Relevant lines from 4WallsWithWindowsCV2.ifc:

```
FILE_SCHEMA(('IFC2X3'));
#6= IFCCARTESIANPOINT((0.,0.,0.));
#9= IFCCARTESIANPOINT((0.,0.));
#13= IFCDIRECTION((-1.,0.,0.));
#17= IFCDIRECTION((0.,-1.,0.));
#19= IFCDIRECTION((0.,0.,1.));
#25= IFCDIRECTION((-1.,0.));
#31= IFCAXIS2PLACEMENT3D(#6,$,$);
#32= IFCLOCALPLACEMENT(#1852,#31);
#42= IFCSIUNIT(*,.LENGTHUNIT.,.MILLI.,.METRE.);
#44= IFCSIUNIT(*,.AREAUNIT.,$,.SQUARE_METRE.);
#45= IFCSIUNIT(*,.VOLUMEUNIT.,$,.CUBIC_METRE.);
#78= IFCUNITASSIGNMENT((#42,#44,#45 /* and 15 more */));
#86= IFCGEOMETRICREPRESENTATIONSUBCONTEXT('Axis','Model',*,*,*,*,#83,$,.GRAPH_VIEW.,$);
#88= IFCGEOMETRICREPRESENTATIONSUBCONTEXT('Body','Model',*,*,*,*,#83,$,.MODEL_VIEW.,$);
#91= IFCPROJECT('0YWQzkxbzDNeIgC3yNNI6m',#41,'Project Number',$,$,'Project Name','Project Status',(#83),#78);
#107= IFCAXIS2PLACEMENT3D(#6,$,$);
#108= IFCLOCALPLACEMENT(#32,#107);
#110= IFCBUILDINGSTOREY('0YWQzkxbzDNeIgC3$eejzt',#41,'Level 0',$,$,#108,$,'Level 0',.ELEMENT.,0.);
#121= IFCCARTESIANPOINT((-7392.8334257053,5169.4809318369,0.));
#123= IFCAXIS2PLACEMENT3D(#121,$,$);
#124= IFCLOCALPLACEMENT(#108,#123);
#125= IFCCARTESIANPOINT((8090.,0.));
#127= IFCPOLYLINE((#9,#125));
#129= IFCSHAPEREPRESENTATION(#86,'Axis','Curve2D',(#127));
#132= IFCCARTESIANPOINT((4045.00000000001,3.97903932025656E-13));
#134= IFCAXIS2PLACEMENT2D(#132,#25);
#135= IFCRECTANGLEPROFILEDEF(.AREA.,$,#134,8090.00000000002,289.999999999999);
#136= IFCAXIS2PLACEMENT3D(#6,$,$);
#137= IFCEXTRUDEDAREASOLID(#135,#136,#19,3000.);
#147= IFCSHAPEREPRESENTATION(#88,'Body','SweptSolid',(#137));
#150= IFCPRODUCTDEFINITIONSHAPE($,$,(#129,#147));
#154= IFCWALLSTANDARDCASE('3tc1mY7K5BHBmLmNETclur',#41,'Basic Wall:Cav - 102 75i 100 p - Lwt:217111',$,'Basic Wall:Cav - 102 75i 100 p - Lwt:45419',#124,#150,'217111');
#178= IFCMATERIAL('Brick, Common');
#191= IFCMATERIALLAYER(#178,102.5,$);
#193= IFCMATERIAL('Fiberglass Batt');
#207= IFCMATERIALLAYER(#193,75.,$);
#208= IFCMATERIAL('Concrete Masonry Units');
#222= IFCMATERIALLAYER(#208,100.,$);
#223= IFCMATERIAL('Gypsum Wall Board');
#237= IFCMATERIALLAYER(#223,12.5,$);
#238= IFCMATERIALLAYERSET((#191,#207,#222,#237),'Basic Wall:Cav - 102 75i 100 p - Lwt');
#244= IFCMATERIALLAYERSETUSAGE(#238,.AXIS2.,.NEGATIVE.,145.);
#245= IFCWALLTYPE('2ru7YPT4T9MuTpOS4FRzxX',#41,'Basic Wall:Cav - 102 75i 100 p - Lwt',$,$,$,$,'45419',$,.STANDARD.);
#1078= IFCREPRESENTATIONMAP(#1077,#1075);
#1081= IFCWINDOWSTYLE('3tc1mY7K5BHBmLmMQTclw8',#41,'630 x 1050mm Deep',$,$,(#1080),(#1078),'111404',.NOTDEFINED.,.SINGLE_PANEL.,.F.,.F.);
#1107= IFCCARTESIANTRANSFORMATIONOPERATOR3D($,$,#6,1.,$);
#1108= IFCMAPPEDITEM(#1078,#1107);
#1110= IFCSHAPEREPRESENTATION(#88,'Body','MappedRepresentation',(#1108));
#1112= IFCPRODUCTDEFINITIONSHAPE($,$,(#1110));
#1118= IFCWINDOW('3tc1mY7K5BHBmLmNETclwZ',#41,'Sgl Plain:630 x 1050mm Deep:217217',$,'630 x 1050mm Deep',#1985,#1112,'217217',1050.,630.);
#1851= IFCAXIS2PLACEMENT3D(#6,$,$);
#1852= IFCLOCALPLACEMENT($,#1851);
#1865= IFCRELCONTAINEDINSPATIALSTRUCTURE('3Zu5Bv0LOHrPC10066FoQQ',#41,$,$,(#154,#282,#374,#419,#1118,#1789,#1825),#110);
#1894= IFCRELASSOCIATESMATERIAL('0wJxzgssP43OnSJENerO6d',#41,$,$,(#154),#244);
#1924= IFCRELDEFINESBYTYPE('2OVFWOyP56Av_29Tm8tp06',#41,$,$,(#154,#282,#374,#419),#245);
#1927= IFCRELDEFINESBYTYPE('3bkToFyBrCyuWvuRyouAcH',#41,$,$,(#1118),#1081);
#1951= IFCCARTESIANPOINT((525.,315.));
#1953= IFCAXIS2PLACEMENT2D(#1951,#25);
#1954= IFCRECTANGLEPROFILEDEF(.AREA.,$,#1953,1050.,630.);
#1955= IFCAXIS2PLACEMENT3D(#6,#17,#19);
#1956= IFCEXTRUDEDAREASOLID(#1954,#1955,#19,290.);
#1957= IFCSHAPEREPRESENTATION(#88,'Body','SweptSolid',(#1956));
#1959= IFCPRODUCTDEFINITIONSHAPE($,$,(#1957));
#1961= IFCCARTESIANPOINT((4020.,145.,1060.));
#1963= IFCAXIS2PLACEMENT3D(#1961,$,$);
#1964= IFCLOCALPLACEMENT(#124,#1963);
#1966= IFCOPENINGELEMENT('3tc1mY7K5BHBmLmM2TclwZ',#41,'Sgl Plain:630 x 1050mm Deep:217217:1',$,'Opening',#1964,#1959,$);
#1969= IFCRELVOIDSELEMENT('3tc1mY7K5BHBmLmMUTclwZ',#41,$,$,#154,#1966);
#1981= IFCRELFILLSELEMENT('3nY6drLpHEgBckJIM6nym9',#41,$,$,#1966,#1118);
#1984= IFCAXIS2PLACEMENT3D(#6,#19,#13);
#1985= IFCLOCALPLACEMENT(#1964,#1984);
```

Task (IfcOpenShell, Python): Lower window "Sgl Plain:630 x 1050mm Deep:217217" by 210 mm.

```python
import numpy as np
import ifcopenshell
import ifcopenshell.api.geometry
import ifcopenshell.util.placement
import ifcopenshell.util.unit

model = ifcopenshell.open("4WallsWithWindowsCV2.ifc")
unit_scale = ifcopenshell.util.unit.calculate_unit_scale(model)

window = model.by_id(1118)
opening = window.FillsVoids[0].RelatingOpeningElement
dz = -0.21 / unit_scale

shift = np.array([0.0, 0.0, dz])
# The window is placed relative to its opening, so it follows when the opening moves.
matrix = ifcopenshell.util.placement.get_local_placement(opening.ObjectPlacement)
matrix[:3, 3] += shift
ifcopenshell.api.geometry.edit_object_placement(
    model, product=opening, matrix=matrix, is_si=False, should_transform_children=True
)

print(f"moved by {dz * unit_scale:+.3f} m")

model.write("4WallsWithWindowsCV2_v2.ifc")
```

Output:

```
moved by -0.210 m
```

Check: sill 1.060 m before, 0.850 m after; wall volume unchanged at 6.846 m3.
